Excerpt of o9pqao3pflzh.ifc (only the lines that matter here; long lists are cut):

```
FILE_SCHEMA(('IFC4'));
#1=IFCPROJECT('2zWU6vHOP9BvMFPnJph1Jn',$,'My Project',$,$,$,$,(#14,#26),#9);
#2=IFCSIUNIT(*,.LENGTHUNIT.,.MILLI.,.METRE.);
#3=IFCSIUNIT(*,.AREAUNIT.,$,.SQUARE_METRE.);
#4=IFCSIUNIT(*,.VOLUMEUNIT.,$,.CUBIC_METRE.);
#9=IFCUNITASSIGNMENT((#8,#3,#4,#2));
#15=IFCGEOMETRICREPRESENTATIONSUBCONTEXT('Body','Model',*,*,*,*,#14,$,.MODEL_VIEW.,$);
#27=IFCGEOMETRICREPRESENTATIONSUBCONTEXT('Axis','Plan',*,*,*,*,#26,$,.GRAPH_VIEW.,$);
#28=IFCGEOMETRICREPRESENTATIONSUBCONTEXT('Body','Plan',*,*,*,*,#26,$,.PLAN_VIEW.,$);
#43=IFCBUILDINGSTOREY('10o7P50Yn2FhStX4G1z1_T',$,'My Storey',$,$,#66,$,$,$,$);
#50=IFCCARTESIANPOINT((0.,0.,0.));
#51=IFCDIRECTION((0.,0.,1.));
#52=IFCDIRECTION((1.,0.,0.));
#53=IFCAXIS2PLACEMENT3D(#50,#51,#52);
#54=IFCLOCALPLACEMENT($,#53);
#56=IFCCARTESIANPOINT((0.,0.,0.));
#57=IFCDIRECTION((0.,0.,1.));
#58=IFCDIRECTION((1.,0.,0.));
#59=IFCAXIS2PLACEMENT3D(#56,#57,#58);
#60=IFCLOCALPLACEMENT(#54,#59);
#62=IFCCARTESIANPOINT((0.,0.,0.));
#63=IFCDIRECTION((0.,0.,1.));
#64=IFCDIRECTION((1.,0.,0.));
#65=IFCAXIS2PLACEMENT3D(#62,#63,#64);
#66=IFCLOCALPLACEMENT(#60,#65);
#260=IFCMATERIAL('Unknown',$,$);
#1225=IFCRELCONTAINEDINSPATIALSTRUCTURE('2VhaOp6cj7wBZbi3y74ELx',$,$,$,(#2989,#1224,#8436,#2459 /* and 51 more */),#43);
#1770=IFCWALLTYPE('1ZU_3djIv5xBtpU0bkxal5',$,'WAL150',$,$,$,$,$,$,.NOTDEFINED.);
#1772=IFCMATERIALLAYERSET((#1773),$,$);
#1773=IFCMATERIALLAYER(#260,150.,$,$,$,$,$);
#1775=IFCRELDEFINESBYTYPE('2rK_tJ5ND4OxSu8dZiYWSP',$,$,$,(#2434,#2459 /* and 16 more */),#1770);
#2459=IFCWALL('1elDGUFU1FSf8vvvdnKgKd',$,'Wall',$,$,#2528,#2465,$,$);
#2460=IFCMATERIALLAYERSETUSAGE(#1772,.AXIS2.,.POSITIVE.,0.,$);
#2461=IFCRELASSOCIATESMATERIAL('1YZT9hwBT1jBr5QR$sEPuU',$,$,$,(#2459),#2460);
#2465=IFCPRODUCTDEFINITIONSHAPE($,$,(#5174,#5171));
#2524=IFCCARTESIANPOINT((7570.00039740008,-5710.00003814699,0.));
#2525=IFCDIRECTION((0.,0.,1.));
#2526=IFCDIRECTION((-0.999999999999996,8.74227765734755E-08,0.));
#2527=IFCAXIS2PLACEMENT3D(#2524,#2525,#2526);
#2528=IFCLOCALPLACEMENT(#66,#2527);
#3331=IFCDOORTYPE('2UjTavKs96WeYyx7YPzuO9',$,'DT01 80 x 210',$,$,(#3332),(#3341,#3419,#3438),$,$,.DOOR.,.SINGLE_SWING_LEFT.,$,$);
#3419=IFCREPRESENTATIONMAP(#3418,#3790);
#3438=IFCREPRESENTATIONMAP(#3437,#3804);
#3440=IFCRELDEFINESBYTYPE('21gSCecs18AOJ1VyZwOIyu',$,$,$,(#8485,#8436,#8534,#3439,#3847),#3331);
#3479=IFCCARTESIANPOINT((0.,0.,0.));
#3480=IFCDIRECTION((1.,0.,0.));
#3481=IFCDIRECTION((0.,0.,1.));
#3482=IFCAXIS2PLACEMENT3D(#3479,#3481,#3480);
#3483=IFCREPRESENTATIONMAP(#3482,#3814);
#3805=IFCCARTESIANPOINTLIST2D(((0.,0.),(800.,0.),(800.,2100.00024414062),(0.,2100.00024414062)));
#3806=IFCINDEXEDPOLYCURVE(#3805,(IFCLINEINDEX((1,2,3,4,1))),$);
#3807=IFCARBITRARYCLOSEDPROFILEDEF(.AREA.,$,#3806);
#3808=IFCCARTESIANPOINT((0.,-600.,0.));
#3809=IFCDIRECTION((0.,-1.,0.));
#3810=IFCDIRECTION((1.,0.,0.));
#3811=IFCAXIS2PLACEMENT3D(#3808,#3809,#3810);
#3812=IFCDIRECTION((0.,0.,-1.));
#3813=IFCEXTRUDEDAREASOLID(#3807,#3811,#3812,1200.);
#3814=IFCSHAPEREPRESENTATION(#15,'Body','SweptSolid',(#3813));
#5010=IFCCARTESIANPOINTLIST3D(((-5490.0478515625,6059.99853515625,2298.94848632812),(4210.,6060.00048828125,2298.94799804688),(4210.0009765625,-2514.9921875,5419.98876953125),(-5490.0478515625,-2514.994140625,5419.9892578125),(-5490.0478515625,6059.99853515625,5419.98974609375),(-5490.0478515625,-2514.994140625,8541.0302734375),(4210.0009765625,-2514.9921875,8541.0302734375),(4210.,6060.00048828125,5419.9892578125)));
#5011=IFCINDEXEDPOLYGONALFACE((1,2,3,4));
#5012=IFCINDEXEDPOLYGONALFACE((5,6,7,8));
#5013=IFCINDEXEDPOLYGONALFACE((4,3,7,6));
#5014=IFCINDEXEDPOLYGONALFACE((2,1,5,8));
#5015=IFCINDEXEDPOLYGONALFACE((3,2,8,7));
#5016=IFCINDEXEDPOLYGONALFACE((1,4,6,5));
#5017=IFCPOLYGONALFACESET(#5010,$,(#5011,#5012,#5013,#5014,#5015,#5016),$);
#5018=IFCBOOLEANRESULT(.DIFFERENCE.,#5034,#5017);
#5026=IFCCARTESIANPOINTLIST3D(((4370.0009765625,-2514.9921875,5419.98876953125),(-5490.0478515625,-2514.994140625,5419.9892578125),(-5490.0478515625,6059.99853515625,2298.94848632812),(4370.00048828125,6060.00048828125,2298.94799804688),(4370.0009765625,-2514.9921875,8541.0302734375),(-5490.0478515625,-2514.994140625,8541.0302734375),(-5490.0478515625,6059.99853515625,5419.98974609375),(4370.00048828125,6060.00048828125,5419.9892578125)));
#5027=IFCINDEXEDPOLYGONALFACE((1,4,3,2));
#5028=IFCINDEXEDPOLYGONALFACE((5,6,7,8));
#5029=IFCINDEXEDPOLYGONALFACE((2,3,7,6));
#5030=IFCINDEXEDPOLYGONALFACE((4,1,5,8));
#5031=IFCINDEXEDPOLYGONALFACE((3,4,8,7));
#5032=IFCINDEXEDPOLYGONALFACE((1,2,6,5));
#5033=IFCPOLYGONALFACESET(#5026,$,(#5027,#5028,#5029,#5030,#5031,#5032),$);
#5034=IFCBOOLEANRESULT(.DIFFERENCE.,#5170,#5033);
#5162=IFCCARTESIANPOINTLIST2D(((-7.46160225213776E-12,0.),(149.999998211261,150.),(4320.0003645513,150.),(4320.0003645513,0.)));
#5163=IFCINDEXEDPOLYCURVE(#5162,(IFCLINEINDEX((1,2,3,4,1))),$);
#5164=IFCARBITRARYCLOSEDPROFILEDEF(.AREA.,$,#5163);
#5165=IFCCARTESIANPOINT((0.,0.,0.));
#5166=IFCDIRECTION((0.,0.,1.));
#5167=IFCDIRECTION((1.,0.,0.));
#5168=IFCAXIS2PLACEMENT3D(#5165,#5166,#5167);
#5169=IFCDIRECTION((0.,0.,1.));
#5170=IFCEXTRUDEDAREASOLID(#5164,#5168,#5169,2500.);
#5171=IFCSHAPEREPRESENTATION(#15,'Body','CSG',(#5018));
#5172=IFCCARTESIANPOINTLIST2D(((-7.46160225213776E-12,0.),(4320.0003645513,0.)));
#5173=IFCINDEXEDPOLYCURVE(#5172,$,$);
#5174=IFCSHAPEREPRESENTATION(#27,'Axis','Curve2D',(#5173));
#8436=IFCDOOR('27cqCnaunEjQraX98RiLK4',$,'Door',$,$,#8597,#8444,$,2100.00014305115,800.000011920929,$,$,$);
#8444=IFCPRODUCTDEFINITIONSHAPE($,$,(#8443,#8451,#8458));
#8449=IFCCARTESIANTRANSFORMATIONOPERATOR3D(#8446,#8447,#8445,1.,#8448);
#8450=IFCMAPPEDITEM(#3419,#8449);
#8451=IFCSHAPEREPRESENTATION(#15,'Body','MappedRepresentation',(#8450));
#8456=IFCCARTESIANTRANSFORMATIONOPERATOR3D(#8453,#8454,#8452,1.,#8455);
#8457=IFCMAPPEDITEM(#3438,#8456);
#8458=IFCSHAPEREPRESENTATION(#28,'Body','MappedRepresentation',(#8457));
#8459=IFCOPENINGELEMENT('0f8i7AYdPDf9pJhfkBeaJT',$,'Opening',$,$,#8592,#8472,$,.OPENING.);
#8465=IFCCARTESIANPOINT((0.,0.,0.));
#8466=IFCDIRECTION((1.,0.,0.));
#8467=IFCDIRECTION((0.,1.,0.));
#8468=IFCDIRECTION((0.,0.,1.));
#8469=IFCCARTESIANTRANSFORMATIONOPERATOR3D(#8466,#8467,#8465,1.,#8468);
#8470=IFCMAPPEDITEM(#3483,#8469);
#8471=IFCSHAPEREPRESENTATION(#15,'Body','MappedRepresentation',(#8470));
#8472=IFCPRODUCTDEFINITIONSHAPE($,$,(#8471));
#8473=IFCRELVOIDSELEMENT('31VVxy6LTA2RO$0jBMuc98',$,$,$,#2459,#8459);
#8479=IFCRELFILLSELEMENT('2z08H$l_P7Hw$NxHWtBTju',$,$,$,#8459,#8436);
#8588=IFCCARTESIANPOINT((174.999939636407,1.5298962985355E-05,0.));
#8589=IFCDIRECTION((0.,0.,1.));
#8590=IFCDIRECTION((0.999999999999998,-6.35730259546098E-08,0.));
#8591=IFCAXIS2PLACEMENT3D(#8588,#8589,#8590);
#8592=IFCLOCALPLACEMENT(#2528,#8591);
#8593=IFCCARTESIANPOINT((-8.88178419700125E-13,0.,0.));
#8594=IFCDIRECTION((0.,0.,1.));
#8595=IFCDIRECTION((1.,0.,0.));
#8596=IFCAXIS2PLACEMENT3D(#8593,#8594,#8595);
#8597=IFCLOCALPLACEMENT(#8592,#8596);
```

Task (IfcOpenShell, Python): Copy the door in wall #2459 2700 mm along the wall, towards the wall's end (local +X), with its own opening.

```python
import ifcopenshell
import ifcopenshell.api.feature
import ifcopenshell.api.geometry
import ifcopenshell.api.root
import ifcopenshell.geom
import ifcopenshell.util.element
import ifcopenshell.util.placement
import ifcopenshell.util.shape

model = ifcopenshell.open("o9pqao3pflzh.ifc")
settings = ifcopenshell.geom.settings()


def volume(element):
    """Net volume in cubic metres, openings subtracted."""
    shape = ifcopenshell.geom.create_shape(settings, element)
    return ifcopenshell.util.shape.get_volume(shape.geometry)


door = model.by_guid("27cqCnaunEjQraX98RiLK4")
opening = door.FillsVoids[0].RelatingOpeningElement
wall = opening.VoidsElements[0].RelatingBuildingElement
before = volume(wall)
shift = ifcopenshell.util.placement.get_local_placement(wall.ObjectPlacement)[:3, 0] * 2700.0

# copy_class copies the void relationship, type, container and properties, but no geometry.
new_opening = ifcopenshell.api.root.copy_class(model, product=opening)
new_opening.Representation = ifcopenshell.util.element.copy_deep(
    model, opening.Representation, exclude=["IfcGeometricRepresentationContext", "IfcRepresentationMap"]
)
new_door = ifcopenshell.api.root.copy_class(model, product=door)
new_door.Representation = ifcopenshell.util.element.copy_deep(
    model, door.Representation, exclude=["IfcGeometricRepresentationContext", "IfcRepresentationMap"]
)
ifcopenshell.api.feature.add_filling(model, opening=new_opening, element=new_door)

for old, new in ((opening, new_opening), (door, new_door)):
    matrix = ifcopenshell.util.placement.get_local_placement(old.ObjectPlacement)
    matrix[:3, 3] += shift
    ifcopenshell.api.geometry.edit_object_placement(model, product=new, matrix=matrix, is_si=False)

after = volume(wall)

print(f"wall volume {before:.3f} -> {after:.3f} m3")

model.write("o9pqao3pflzh-out.ifc")
```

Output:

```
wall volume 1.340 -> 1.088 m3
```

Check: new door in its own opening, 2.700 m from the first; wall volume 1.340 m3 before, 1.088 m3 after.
